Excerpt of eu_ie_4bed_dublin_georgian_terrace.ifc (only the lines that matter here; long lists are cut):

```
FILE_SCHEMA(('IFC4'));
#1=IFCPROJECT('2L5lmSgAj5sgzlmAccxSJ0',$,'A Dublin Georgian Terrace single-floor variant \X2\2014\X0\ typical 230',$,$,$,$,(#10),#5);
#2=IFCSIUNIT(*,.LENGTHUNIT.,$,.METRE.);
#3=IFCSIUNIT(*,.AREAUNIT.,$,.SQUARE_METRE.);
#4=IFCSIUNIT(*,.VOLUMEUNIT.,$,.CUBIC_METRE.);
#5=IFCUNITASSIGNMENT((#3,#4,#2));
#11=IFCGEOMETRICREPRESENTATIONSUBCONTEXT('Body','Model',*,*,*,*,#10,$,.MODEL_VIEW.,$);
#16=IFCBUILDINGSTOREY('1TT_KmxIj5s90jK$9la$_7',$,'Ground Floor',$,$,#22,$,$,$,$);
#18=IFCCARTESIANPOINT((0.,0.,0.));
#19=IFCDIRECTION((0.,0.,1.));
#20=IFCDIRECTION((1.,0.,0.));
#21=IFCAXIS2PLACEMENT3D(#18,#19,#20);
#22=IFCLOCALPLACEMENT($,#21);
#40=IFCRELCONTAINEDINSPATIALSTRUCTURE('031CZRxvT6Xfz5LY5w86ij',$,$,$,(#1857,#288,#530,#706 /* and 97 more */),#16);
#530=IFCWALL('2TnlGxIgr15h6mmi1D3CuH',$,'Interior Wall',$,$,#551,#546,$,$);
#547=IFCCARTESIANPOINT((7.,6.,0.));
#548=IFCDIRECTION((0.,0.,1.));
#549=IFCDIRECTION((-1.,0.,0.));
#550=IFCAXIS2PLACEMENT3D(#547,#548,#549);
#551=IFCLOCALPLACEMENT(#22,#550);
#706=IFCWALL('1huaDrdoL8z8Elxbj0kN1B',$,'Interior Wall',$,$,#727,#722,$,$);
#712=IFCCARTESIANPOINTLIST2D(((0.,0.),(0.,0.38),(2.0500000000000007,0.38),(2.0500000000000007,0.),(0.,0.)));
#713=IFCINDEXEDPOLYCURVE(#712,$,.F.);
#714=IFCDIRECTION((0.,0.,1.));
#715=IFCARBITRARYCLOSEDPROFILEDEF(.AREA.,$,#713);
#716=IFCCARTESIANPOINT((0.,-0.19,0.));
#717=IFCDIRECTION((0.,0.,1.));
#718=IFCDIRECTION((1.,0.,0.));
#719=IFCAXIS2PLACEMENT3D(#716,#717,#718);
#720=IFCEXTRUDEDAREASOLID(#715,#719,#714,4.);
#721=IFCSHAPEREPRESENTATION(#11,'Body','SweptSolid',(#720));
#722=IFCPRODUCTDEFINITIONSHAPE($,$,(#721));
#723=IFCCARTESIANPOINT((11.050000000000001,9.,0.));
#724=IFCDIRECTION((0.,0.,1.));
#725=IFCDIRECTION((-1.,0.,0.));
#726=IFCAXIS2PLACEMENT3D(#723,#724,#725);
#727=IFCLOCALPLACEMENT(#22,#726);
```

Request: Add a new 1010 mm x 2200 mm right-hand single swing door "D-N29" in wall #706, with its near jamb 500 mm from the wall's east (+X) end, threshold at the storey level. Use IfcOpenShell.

```python
import numpy as np
import ifcopenshell
import ifcopenshell.api.feature
import ifcopenshell.api.geometry
import ifcopenshell.api.root
import ifcopenshell.api.spatial
import ifcopenshell.geom
import ifcopenshell.util.element
import ifcopenshell.util.placement
import ifcopenshell.util.representation
import ifcopenshell.util.shape
import ifcopenshell.util.unit

model = ifcopenshell.open("eu_ie_4bed_dublin_georgian_terrace.ifc")
unit_scale = ifcopenshell.util.unit.calculate_unit_scale(model)
settings = ifcopenshell.geom.settings()


def volume(element):
    """Net volume in cubic metres, openings subtracted."""
    shape = ifcopenshell.geom.create_shape(settings, element)
    return ifcopenshell.util.shape.get_volume(shape.geometry)


wall = model.by_guid("1huaDrdoL8z8Elxbj0kN1B")
storey = ifcopenshell.util.element.get_container(wall, ifc_class="IfcBuildingStorey")
context = ifcopenshell.util.representation.get_context(model, "Model", "Body", "MODEL_VIEW")
before = volume(wall)

width, height, from_end, sill = 1.01, 2.2, 0.5, 0.0  # metres

# The wall runs along its own X axis, and the end named is its -X end.
wall_shape = ifcopenshell.geom.create_shape(settings, wall)
x, y, z = ifcopenshell.util.shape.get_vertices(wall_shape.geometry).T
start = x.min() + from_end
face, thickness = float(y.min()), float(y.max() - y.min())
wall_matrix = ifcopenshell.util.placement.get_local_placement(wall.ObjectPlacement)
level = ifcopenshell.util.placement.get_local_placement(storey.ObjectPlacement)[2, 3]


def in_wall(x, y):
    """Placement at x, y metres in the wall's axes, at sill height."""
    matrix = wall_matrix.copy()
    matrix[:, 3] = wall_matrix @ np.array([x / unit_scale, y / unit_scale, 0.0, 1.0])
    matrix[2, 3] = level + sill / unit_scale
    return matrix


# Opening: a box that overshoots both wall faces by 50 mm.
opening = ifcopenshell.api.root.create_entity(model, ifc_class="IfcOpeningElement", predefined_type="OPENING")
box = ifcopenshell.api.geometry.add_wall_representation(
    model, context=context, length=width, height=height, thickness=thickness + 0.1
)
ifcopenshell.api.geometry.assign_representation(model, product=opening, representation=box)
ifcopenshell.api.geometry.edit_object_placement(model, product=opening, matrix=in_wall(start, face - 0.05), is_si=False)
ifcopenshell.api.feature.add_feature(model, feature=opening, element=wall)

door = ifcopenshell.api.root.create_entity(model, ifc_class="IfcDoor", name="D-N29", predefined_type="DOOR")
door.OverallWidth, door.OverallHeight = width / unit_scale, height / unit_scale
door.OperationType = "SINGLE_SWING_RIGHT"
body = ifcopenshell.api.geometry.add_door_representation(
    model,
    context=context,
    overall_width=door.OverallWidth,
    overall_height=door.OverallHeight,
    operation_type="SINGLE_SWING_RIGHT",
    lining_properties={"LiningDepth": thickness / unit_scale, "ThresholdDepth": thickness / unit_scale},
)
ifcopenshell.api.geometry.assign_representation(model, product=door, representation=body)
ifcopenshell.api.spatial.assign_container(model, products=[door], relating_structure=storey)
ifcopenshell.api.feature.add_filling(model, opening=opening, element=door)

# The lining spans the wall, so the door starts at the wall face.
ifcopenshell.api.geometry.edit_object_placement(model, product=door, matrix=in_wall(start, face), is_si=False)

after = volume(wall)

print(f"wall volume {before:.3f} -> {after:.3f} m3")

model.write("eu_ie_4bed_dublin_georgian_terrace_updated.ifc")
```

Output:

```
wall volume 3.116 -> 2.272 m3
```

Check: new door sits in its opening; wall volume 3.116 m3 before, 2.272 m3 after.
